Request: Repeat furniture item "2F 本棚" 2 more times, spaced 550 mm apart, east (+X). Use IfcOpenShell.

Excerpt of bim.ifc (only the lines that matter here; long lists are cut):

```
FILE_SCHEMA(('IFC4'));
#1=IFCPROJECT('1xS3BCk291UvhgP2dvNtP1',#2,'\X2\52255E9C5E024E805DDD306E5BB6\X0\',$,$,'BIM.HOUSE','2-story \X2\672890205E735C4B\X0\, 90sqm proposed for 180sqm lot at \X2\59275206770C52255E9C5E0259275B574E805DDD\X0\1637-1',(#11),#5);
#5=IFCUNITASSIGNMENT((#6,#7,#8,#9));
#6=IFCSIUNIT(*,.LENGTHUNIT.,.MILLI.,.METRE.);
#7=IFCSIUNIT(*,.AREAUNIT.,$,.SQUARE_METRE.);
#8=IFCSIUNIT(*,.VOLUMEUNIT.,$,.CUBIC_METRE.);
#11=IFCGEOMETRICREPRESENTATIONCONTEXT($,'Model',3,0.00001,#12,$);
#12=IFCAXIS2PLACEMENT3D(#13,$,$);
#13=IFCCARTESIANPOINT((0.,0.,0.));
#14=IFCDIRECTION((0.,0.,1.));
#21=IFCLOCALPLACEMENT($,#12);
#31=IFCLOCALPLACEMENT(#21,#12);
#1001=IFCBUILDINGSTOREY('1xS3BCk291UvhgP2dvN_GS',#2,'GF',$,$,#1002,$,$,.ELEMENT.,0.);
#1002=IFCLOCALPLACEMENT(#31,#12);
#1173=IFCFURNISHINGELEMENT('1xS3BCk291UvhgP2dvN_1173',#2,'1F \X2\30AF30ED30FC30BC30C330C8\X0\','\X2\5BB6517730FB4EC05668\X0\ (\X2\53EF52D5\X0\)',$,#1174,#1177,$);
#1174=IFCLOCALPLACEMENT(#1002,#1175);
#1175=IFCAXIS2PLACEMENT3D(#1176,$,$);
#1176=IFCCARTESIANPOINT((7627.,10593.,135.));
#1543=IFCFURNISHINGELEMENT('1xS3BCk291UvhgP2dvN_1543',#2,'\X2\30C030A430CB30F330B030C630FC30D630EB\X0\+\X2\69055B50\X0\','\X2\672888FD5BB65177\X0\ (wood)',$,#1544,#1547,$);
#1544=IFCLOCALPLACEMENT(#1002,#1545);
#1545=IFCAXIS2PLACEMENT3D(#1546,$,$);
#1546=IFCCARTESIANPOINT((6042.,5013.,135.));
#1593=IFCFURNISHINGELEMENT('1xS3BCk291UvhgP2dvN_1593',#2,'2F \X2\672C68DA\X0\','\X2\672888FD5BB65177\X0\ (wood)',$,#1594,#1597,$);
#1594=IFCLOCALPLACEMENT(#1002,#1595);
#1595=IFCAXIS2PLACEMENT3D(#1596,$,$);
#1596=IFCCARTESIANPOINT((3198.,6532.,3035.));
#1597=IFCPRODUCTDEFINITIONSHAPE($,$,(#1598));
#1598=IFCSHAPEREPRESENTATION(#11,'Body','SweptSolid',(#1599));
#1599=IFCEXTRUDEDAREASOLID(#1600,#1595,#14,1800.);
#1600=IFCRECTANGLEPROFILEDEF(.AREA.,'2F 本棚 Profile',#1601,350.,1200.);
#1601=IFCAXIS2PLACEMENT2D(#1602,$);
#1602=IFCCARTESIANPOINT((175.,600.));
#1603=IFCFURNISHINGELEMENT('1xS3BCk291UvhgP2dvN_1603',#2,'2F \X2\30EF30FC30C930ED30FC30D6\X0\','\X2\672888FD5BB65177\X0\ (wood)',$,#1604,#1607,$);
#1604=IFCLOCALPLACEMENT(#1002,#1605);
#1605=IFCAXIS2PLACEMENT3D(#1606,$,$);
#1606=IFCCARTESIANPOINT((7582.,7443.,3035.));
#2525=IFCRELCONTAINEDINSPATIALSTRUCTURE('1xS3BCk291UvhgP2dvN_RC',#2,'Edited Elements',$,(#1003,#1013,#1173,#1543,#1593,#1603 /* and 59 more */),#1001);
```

```python
import numpy as np
import ifcopenshell
import ifcopenshell.api.geometry
import ifcopenshell.api.root
import ifcopenshell.util.element
import ifcopenshell.util.placement
import ifcopenshell.util.unit

model = ifcopenshell.open("bim.ifc")
unit_scale = ifcopenshell.util.unit.calculate_unit_scale(model)


def reuse_history(source, copy):
    """copy_class also copies each property set's owner history, people and application; keep the originals."""
    for rel in copy.IsDefinedBy:
        if rel.is_a("IfcRelDefinesByProperties") and (history := rel.RelatingPropertyDefinition.OwnerHistory):
            rel.RelatingPropertyDefinition.OwnerHistory = source.OwnerHistory
            ifcopenshell.util.element.remove_deep2(model, history)


source = model.by_id(1593)
base = ifcopenshell.util.placement.get_local_placement(source.ObjectPlacement)
step = np.array([1.0, 0.0, 0.0]) * 0.55 / unit_scale

for i in range(1, 3):
    copy = ifcopenshell.api.root.copy_class(model, product=source)
    copy.Representation = ifcopenshell.util.element.copy_deep(
        model, source.Representation, exclude=["IfcGeometricRepresentationContext", "IfcRepresentationMap"]
    )
    reuse_history(source, copy)
    matrix = base.copy()
    matrix[:3, 3] += i * step
    print("added at", matrix[:3, 3].round(3) + 0.0)
    ifcopenshell.api.geometry.edit_object_placement(model, product=copy, matrix=matrix, is_si=False)

model.write("bim-out.ifc")
```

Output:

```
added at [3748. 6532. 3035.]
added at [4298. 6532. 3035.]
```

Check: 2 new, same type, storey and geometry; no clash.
